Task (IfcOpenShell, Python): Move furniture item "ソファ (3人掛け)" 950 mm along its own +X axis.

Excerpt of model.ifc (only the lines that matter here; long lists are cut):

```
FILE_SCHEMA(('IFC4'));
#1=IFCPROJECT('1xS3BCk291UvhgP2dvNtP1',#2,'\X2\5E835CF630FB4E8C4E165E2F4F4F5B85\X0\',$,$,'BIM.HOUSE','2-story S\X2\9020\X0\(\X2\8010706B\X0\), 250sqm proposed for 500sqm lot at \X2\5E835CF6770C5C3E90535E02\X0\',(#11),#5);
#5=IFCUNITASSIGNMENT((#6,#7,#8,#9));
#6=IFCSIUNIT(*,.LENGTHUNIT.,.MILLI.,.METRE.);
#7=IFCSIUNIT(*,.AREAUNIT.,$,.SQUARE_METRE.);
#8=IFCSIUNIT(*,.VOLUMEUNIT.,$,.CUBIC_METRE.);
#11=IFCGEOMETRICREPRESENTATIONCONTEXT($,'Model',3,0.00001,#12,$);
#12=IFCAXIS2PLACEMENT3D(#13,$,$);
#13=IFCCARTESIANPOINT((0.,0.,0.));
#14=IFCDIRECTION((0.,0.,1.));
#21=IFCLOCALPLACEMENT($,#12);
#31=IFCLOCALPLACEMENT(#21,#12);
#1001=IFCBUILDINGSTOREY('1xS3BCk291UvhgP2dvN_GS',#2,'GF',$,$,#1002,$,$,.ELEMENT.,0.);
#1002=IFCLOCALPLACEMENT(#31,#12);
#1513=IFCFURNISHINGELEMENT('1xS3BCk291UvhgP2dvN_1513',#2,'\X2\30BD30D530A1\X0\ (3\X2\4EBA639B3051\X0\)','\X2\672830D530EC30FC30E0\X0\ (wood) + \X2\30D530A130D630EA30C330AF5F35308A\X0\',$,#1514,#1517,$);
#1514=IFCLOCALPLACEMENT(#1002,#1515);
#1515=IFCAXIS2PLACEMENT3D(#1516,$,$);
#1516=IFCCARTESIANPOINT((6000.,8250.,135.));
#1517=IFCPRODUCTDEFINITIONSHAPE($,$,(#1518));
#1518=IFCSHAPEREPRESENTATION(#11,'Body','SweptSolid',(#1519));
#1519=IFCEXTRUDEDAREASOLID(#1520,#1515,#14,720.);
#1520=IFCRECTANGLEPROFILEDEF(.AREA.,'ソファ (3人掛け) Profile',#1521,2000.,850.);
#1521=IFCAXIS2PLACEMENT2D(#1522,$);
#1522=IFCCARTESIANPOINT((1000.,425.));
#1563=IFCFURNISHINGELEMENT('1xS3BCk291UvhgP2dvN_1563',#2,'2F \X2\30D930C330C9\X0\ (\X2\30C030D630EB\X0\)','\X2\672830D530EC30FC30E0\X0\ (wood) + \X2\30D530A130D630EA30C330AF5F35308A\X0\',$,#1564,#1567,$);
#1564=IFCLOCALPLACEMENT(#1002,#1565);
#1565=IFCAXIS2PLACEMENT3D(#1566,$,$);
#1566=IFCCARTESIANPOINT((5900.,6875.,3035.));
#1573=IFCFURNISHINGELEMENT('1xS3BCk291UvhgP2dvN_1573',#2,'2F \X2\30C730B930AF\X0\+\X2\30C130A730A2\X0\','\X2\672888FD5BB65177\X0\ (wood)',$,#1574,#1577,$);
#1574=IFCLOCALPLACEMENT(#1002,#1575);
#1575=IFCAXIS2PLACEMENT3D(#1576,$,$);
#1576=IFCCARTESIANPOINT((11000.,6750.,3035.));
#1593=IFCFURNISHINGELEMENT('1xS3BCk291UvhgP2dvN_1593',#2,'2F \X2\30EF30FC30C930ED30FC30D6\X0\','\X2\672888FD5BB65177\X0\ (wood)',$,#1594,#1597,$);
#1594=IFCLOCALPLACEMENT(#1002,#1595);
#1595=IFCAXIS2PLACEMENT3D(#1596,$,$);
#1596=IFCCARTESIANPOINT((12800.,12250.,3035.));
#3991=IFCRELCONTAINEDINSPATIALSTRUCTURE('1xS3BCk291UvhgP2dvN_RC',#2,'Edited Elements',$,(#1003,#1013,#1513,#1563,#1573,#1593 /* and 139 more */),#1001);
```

```python
import ifcopenshell
import ifcopenshell.api.geometry
import ifcopenshell.util.placement
import ifcopenshell.util.unit

model = ifcopenshell.open("model.ifc")
unit_scale = ifcopenshell.util.unit.calculate_unit_scale(model)

item = model.by_guid("1xS3BCk291UvhgP2dvN_1513")
matrix = ifcopenshell.util.placement.get_local_placement(item.ObjectPlacement)
matrix[:3, 3] += matrix[:3, 0] * 0.95 / unit_scale
ifcopenshell.api.geometry.edit_object_placement(model, product=item, matrix=matrix, is_si=False)

print(ifcopenshell.util.placement.get_local_placement(item.ObjectPlacement).round(3) + 0.0)

model.write("model-out.ifc")
```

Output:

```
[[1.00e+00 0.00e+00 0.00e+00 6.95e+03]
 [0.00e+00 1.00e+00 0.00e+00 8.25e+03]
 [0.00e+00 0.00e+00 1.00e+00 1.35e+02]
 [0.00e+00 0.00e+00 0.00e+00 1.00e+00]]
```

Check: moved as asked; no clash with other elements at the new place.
